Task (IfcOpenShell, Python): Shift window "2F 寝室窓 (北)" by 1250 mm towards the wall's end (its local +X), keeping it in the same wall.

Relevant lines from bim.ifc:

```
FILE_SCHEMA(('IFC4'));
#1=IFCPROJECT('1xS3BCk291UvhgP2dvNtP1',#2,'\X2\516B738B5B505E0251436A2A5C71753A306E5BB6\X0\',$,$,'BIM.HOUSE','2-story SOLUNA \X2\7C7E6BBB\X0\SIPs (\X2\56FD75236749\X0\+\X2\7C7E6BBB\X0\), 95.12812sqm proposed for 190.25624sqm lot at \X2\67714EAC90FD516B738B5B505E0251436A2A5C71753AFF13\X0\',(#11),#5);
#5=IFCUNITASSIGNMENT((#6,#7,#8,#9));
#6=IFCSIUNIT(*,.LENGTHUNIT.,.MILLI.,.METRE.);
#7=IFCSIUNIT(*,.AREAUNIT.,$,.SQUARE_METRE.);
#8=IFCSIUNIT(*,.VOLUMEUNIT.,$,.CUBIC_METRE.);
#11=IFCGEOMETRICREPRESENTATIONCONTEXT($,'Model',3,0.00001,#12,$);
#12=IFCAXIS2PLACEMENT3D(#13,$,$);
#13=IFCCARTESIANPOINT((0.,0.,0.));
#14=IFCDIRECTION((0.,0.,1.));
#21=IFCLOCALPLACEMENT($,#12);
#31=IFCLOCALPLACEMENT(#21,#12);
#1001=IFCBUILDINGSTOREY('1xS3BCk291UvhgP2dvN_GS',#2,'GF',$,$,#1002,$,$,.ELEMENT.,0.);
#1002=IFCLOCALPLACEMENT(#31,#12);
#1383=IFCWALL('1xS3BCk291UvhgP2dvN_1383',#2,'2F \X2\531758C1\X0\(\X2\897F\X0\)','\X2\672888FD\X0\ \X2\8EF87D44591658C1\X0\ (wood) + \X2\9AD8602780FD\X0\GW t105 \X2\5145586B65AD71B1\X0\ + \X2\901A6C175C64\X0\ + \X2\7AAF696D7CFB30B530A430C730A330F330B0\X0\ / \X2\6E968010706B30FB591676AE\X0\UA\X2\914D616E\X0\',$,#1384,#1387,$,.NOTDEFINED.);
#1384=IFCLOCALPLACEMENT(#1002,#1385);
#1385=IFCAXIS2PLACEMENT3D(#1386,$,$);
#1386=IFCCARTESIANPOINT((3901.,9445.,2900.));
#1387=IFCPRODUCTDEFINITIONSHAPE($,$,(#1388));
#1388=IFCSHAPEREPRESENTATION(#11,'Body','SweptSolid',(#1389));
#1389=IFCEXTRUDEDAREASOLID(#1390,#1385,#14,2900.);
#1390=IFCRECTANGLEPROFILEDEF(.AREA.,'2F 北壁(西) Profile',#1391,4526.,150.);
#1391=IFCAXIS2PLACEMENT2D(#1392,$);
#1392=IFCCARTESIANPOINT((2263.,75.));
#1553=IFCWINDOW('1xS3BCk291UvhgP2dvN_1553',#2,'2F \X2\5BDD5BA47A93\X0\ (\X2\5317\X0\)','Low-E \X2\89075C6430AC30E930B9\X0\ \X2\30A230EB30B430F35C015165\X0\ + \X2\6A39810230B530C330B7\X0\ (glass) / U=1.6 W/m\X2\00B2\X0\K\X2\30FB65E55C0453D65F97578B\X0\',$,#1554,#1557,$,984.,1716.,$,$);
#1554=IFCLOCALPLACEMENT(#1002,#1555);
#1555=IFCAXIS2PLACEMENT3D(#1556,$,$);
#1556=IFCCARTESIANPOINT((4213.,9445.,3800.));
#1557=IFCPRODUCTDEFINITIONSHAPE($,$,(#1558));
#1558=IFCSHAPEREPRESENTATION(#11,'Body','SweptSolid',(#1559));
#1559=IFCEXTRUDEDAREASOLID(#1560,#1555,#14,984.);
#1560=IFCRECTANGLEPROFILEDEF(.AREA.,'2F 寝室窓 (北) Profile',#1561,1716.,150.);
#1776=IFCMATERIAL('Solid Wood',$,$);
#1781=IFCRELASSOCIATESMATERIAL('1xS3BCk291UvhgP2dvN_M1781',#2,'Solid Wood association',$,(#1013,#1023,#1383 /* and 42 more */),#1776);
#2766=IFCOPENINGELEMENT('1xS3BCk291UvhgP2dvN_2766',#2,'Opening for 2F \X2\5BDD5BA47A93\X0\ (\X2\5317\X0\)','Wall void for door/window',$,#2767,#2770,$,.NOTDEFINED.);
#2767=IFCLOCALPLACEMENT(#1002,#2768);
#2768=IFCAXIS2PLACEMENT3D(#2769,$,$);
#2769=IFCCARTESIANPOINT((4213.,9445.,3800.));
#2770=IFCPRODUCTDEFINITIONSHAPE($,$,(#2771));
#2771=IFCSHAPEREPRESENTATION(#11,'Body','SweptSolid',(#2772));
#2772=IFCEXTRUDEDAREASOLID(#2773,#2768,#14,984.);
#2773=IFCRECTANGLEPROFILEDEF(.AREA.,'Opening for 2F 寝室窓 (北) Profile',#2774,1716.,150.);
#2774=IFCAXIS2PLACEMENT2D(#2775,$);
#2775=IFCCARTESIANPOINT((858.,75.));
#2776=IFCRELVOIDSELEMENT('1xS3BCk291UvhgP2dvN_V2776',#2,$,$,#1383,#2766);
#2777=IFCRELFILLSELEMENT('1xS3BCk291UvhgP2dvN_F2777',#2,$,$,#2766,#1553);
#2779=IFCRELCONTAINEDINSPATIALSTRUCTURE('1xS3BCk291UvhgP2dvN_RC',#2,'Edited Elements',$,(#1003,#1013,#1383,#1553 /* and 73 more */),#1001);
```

```python
import ifcopenshell
import ifcopenshell.api.geometry
import ifcopenshell.util.placement

model = ifcopenshell.open("bim.ifc")

window = model.by_guid("1xS3BCk291UvhgP2dvN_1553")
opening = window.FillsVoids[0].RelatingOpeningElement
wall = opening.VoidsElements[0].RelatingBuildingElement

wall_matrix = ifcopenshell.util.placement.get_local_placement(wall.ObjectPlacement)
shift = wall_matrix[:3, 0] * 1250.0
before = ifcopenshell.util.placement.get_local_placement(window.ObjectPlacement)[:3, 3].copy()

# The window is not placed relative to its opening, so move both.
for product in (opening, window):
    matrix = ifcopenshell.util.placement.get_local_placement(product.ObjectPlacement)
    matrix[:3, 3] += shift
    ifcopenshell.api.geometry.edit_object_placement(model, product=product, matrix=matrix, is_si=False)

after = ifcopenshell.util.placement.get_local_placement(window.ObjectPlacement)[:3, 3]
print("window moved by", (after - before).round(3) + 0.0)

model.write("bim_updated.ifc")
```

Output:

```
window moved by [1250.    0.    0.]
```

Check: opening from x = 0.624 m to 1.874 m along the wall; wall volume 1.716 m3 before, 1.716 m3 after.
